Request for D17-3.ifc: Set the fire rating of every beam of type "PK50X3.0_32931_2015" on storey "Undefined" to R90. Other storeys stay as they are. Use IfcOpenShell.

First a look at what the model holds.

```python
import ifcopenshell
import ifcopenshell.util.element

model = ifcopenshell.open("D17-3.ifc")
print(model.schema)
storey = next(s for s in model.by_type("IfcBuildingStorey") if s.Name == "Undefined")
beams = [e for e in ifcopenshell.util.element.get_decomposition(storey) if e.is_a("IfcBeam")]
seen = {}
for e in beams:
    element_type = ifcopenshell.util.element.get_type(e)
    key = (element_type.Name if element_type != e and element_type else None, ifcopenshell.util.element.get_pset(e, "Pset_BeamCommon", "FireRating"))
    seen[key] = seen.get(key, 0) + 1
for (name, value), count in sorted(seen.items(), key=str):
    print(count, "x", name, "|", value)
```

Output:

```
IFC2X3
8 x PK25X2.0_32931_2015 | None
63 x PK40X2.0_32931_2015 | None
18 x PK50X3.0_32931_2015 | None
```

```python
import ifcopenshell
import ifcopenshell.api.pset
import ifcopenshell.util.element

model = ifcopenshell.open("D17-3.ifc")

storey = next(s for s in model.by_type("IfcBuildingStorey") if s.Name == "Undefined")
beams = [e for e in ifcopenshell.util.element.get_decomposition(storey) if e.is_a("IfcBeam")]

count = 0
for e in beams:
    element_type = ifcopenshell.util.element.get_type(e)
    if element_type in (None, e) or element_type.Name != "PK50X3.0_32931_2015":
        continue
    found = ifcopenshell.util.element.get_pset(e, "Pset_BeamCommon", should_inherit=False)
    if found:
        pset = model.by_id(found["id"])
        if len(ifcopenshell.util.element.get_elements_by_pset(pset)) > 1:
            pset = ifcopenshell.api.pset.unshare_pset(model, products=[e], pset=pset)[0]
    else:
        pset = ifcopenshell.api.pset.add_pset(model, product=e, name="Pset_BeamCommon")
    ifcopenshell.api.pset.edit_pset(model, pset=pset, properties={"FireRating": "R90"})
    count += 1

print(count, "beams updated")

model.write("D17-3_updated.ifc")
```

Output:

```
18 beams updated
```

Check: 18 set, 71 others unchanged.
